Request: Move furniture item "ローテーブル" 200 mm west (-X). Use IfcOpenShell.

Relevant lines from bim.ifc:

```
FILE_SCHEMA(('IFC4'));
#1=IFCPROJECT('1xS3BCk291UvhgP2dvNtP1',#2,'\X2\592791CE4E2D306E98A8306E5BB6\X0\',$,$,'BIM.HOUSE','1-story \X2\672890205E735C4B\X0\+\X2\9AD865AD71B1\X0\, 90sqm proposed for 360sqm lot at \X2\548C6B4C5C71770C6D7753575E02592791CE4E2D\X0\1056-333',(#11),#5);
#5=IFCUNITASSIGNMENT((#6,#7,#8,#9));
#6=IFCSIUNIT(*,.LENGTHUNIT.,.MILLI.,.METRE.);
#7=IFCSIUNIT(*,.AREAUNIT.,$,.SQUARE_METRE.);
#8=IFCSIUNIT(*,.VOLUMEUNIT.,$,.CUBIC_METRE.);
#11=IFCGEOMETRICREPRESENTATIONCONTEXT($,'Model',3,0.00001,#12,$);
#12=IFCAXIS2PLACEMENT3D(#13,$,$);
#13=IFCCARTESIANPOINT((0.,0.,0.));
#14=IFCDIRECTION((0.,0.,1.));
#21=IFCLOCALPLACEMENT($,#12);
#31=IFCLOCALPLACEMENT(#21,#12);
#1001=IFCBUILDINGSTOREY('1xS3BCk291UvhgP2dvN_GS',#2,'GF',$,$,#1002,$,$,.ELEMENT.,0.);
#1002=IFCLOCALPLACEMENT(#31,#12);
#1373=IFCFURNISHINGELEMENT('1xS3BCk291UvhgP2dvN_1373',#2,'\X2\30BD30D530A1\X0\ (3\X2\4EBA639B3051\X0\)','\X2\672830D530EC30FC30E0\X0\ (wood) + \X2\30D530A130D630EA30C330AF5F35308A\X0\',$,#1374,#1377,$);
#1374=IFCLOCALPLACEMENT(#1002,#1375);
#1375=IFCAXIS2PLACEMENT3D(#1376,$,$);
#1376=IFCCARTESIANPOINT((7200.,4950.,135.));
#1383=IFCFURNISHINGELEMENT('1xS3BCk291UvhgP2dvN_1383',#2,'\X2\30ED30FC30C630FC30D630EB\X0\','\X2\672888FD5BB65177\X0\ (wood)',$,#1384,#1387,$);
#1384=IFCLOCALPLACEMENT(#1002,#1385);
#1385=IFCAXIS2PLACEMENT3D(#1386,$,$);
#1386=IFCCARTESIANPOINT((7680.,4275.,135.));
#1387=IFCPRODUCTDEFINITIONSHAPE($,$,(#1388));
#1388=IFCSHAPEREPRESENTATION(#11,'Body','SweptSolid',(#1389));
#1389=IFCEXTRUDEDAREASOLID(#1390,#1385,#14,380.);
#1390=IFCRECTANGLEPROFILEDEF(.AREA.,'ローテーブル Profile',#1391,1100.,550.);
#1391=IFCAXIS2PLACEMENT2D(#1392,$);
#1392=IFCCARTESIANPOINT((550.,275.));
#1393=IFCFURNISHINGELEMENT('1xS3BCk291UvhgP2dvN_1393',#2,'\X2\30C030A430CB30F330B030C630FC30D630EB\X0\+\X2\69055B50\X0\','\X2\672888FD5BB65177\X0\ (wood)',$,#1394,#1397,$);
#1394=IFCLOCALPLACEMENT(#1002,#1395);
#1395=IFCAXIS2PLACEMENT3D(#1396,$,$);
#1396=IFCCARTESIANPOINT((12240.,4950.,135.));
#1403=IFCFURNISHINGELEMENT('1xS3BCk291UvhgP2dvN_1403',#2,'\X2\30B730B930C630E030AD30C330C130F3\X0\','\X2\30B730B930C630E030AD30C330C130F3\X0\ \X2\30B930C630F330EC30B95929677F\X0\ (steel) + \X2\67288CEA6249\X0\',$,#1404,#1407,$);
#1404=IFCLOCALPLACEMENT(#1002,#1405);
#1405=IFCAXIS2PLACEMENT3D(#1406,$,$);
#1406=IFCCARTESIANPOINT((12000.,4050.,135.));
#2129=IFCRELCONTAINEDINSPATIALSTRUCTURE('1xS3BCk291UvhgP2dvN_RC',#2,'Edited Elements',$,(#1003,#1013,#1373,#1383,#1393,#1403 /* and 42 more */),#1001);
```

```python
import ifcopenshell
import ifcopenshell.api.geometry
import ifcopenshell.util.placement
import ifcopenshell.util.unit

model = ifcopenshell.open("bim.ifc")
unit_scale = ifcopenshell.util.unit.calculate_unit_scale(model)

item = model.by_guid("1xS3BCk291UvhgP2dvN_1383")
matrix = ifcopenshell.util.placement.get_local_placement(item.ObjectPlacement)
matrix[0, 3] -= 0.2 / unit_scale
ifcopenshell.api.geometry.edit_object_placement(model, product=item, matrix=matrix, is_si=False)

print(ifcopenshell.util.placement.get_local_placement(item.ObjectPlacement).round(3) + 0.0)

model.write("bim_edited.ifc")
```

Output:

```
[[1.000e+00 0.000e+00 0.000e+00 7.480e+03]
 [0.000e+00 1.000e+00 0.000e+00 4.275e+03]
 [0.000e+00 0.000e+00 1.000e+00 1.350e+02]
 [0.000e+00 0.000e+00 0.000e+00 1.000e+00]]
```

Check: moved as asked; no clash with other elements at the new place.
